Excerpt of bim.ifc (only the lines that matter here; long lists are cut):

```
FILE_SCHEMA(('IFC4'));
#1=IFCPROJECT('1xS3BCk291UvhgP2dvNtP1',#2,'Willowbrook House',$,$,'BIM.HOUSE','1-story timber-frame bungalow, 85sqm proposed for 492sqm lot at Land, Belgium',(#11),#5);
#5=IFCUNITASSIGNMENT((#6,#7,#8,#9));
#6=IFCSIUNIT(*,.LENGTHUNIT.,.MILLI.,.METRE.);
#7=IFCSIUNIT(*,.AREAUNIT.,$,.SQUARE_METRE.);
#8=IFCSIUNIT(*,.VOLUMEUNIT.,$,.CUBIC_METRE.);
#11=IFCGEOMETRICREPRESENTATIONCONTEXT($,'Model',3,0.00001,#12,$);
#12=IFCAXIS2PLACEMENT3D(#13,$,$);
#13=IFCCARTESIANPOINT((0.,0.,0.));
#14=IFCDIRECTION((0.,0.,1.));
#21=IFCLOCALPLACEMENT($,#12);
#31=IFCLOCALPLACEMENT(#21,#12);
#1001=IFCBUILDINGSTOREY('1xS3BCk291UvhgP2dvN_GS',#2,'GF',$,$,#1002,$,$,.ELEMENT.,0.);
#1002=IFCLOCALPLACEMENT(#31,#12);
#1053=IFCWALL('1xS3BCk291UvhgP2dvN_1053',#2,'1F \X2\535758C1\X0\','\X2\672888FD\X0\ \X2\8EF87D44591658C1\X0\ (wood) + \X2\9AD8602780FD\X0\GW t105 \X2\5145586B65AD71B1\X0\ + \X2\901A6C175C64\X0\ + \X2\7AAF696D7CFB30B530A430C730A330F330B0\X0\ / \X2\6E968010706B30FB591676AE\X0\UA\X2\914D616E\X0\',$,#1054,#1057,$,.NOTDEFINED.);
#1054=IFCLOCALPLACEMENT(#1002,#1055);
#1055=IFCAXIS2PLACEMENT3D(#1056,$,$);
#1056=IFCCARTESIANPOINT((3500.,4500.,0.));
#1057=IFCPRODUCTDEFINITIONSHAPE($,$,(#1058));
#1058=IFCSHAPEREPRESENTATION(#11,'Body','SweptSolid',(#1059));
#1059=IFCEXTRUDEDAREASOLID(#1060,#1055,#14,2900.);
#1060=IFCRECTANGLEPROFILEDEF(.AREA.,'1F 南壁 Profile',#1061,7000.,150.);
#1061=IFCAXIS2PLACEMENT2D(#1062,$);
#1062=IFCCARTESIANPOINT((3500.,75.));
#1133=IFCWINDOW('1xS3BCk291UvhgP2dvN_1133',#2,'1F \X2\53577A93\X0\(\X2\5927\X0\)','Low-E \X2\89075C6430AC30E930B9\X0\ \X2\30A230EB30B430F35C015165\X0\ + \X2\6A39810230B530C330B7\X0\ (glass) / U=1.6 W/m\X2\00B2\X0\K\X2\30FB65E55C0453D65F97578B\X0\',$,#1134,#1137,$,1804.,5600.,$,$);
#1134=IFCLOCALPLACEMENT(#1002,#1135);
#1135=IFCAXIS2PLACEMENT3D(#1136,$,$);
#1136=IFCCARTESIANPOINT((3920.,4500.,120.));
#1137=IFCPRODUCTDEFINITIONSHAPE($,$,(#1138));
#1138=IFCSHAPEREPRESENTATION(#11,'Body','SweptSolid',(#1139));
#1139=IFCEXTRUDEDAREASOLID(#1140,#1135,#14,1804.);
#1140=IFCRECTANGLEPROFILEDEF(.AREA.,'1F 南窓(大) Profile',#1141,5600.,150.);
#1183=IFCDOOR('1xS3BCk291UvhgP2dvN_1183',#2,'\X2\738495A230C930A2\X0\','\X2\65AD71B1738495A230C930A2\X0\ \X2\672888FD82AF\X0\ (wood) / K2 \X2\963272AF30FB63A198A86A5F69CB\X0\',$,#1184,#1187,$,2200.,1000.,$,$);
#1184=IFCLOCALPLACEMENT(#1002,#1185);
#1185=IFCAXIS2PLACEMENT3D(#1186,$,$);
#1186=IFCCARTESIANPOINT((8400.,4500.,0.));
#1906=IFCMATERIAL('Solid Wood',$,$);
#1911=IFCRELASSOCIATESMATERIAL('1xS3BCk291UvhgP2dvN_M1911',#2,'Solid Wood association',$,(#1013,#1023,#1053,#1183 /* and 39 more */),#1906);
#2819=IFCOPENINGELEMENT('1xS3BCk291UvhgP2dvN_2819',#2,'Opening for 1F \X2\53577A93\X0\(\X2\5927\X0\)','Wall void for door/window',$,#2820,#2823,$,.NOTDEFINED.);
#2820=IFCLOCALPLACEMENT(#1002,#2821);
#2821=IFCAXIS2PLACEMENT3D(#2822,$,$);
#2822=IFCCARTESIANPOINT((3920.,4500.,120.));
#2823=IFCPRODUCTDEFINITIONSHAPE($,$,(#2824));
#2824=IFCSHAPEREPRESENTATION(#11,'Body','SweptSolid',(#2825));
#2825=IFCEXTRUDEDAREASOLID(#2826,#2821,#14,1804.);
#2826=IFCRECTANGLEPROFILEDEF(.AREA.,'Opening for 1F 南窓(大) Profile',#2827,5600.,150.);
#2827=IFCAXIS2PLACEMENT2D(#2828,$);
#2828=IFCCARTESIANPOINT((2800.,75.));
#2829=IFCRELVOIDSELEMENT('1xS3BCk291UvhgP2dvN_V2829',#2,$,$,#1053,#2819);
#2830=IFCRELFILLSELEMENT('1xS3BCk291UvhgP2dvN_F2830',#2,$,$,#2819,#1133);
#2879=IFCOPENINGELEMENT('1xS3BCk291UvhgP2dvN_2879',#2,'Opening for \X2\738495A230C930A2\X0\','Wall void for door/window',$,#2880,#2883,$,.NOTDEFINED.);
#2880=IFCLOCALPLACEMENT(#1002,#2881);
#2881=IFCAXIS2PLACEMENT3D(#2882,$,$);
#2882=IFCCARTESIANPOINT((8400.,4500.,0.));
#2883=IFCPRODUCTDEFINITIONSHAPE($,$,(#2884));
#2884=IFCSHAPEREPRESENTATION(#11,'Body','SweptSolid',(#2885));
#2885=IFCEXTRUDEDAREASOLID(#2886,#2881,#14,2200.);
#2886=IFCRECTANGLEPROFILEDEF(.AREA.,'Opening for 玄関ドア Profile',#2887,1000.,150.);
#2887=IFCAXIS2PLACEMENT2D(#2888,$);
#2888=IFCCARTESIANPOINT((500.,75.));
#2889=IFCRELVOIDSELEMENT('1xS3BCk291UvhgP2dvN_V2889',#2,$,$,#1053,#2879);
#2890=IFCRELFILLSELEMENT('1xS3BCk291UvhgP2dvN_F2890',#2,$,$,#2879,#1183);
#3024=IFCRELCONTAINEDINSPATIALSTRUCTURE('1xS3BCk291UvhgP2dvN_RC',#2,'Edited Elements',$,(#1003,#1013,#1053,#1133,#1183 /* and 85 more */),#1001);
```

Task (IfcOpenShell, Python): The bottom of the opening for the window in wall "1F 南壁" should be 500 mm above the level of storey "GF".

```python
import numpy as np
import ifcopenshell
import ifcopenshell.api.geometry
import ifcopenshell.geom
import ifcopenshell.util.element
import ifcopenshell.util.placement
import ifcopenshell.util.shape
import ifcopenshell.util.unit

model = ifcopenshell.open("bim.ifc")
unit_scale = ifcopenshell.util.unit.calculate_unit_scale(model)

window = model.by_guid("1xS3BCk291UvhgP2dvN_1133")
opening = window.FillsVoids[0].RelatingOpeningElement
storey = ifcopenshell.util.element.get_container(window, ifc_class="IfcBuildingStorey")
level = ifcopenshell.util.placement.get_local_placement(storey.ObjectPlacement)[2, 3]

# The opening's origin need not be at the sill, so measure its lowest point.
shape = ifcopenshell.geom.create_shape(ifcopenshell.geom.settings(), opening)
bottom = ifcopenshell.util.shape.get_shape_bottom_elevation(shape, shape.geometry) / unit_scale
dz = level + 500.0 - bottom

shift = np.array([0.0, 0.0, dz])
# The window is not placed relative to its opening, so move both.
for product in (opening, window):
    matrix = ifcopenshell.util.placement.get_local_placement(product.ObjectPlacement)
    matrix[:3, 3] += shift
    ifcopenshell.api.geometry.edit_object_placement(model, product=product, matrix=matrix, is_si=False)

print(f"moved by {dz * unit_scale:+.3f} m")

model.write("bim_updated.ifc")
```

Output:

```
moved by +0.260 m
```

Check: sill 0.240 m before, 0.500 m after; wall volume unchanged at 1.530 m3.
